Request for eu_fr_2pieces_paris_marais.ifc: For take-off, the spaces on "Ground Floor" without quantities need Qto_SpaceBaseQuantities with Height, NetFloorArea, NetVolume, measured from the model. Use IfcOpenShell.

First a look at what the model holds.

```python
import ifcopenshell
import ifcopenshell.util.element
import ifcopenshell.util.unit

model = ifcopenshell.open("eu_fr_2pieces_paris_marais.ifc")
print(model.schema)
for unit_type in ("LENGTHUNIT", "AREAUNIT", "VOLUMEUNIT"):
    print(unit_type, ifcopenshell.util.unit.calculate_unit_scale(model, unit_type))
storey = next(s for s in model.by_type("IfcBuildingStorey") if s.Name == "Ground Floor")
spaces = [e for e in ifcopenshell.util.element.get_decomposition(storey) if e.is_a("IfcSpace")]
for e in sorted(spaces, key=lambda e: e.id()):
    print(e.id(), e.is_a(), e.Name, list(ifcopenshell.util.element.get_psets(e, qtos_only=True)), sep=" | ")
```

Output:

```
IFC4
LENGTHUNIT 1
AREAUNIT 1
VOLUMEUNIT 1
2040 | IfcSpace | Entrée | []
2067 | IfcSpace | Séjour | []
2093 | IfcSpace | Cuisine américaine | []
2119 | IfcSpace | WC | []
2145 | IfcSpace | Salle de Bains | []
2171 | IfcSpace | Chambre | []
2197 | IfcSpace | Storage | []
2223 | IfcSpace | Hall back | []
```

```python
import ifcopenshell
import ifcopenshell.api.pset
import ifcopenshell.geom
import ifcopenshell.util.element
import ifcopenshell.util.shape
import ifcopenshell.util.unit

model = ifcopenshell.open("eu_fr_2pieces_paris_marais.ifc")
unit_scale = ifcopenshell.util.unit.calculate_unit_scale(model)
area_scale = ifcopenshell.util.unit.calculate_unit_scale(model, "AREAUNIT")
volume_scale = ifcopenshell.util.unit.calculate_unit_scale(model, "VOLUMEUNIT")
settings = ifcopenshell.geom.settings()

storey = next(s for s in model.by_type("IfcBuildingStorey") if s.Name == "Ground Floor")
spaces = [e for e in ifcopenshell.util.element.get_decomposition(storey) if e.is_a("IfcSpace")]

for e in sorted(spaces, key=lambda e: e.id()):
    if ifcopenshell.util.element.get_psets(e, qtos_only=True, should_inherit=False):
        continue
    # Geometry comes back in metres, in the element's own axes.
    shape = ifcopenshell.geom.create_shape(settings, e)
    values = {
        "Height": ifcopenshell.util.shape.get_z(shape.geometry) / unit_scale,
        "NetFloorArea": ifcopenshell.util.shape.get_footprint_area(shape.geometry) / area_scale,
        "NetVolume": ifcopenshell.util.shape.get_volume(shape.geometry) / volume_scale,
    }
    qto = ifcopenshell.api.pset.add_qto(model, product=e, name="Qto_SpaceBaseQuantities")
    ifcopenshell.api.pset.edit_qto(model, qto=qto, properties=values)
    print(e.id(), {k: round(v, 3) for k, v in values.items()})

model.write("eu_fr_2pieces_paris_marais-out.ifc")
```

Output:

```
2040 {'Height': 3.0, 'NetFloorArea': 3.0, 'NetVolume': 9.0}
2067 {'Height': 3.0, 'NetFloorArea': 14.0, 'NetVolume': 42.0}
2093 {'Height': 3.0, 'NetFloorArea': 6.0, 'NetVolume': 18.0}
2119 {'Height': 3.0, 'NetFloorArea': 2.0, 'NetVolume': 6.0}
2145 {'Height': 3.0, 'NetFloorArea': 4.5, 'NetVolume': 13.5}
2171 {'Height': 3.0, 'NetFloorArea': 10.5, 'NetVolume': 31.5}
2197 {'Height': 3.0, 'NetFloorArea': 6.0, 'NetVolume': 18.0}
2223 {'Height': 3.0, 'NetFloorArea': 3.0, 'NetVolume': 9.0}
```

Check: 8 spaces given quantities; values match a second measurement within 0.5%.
